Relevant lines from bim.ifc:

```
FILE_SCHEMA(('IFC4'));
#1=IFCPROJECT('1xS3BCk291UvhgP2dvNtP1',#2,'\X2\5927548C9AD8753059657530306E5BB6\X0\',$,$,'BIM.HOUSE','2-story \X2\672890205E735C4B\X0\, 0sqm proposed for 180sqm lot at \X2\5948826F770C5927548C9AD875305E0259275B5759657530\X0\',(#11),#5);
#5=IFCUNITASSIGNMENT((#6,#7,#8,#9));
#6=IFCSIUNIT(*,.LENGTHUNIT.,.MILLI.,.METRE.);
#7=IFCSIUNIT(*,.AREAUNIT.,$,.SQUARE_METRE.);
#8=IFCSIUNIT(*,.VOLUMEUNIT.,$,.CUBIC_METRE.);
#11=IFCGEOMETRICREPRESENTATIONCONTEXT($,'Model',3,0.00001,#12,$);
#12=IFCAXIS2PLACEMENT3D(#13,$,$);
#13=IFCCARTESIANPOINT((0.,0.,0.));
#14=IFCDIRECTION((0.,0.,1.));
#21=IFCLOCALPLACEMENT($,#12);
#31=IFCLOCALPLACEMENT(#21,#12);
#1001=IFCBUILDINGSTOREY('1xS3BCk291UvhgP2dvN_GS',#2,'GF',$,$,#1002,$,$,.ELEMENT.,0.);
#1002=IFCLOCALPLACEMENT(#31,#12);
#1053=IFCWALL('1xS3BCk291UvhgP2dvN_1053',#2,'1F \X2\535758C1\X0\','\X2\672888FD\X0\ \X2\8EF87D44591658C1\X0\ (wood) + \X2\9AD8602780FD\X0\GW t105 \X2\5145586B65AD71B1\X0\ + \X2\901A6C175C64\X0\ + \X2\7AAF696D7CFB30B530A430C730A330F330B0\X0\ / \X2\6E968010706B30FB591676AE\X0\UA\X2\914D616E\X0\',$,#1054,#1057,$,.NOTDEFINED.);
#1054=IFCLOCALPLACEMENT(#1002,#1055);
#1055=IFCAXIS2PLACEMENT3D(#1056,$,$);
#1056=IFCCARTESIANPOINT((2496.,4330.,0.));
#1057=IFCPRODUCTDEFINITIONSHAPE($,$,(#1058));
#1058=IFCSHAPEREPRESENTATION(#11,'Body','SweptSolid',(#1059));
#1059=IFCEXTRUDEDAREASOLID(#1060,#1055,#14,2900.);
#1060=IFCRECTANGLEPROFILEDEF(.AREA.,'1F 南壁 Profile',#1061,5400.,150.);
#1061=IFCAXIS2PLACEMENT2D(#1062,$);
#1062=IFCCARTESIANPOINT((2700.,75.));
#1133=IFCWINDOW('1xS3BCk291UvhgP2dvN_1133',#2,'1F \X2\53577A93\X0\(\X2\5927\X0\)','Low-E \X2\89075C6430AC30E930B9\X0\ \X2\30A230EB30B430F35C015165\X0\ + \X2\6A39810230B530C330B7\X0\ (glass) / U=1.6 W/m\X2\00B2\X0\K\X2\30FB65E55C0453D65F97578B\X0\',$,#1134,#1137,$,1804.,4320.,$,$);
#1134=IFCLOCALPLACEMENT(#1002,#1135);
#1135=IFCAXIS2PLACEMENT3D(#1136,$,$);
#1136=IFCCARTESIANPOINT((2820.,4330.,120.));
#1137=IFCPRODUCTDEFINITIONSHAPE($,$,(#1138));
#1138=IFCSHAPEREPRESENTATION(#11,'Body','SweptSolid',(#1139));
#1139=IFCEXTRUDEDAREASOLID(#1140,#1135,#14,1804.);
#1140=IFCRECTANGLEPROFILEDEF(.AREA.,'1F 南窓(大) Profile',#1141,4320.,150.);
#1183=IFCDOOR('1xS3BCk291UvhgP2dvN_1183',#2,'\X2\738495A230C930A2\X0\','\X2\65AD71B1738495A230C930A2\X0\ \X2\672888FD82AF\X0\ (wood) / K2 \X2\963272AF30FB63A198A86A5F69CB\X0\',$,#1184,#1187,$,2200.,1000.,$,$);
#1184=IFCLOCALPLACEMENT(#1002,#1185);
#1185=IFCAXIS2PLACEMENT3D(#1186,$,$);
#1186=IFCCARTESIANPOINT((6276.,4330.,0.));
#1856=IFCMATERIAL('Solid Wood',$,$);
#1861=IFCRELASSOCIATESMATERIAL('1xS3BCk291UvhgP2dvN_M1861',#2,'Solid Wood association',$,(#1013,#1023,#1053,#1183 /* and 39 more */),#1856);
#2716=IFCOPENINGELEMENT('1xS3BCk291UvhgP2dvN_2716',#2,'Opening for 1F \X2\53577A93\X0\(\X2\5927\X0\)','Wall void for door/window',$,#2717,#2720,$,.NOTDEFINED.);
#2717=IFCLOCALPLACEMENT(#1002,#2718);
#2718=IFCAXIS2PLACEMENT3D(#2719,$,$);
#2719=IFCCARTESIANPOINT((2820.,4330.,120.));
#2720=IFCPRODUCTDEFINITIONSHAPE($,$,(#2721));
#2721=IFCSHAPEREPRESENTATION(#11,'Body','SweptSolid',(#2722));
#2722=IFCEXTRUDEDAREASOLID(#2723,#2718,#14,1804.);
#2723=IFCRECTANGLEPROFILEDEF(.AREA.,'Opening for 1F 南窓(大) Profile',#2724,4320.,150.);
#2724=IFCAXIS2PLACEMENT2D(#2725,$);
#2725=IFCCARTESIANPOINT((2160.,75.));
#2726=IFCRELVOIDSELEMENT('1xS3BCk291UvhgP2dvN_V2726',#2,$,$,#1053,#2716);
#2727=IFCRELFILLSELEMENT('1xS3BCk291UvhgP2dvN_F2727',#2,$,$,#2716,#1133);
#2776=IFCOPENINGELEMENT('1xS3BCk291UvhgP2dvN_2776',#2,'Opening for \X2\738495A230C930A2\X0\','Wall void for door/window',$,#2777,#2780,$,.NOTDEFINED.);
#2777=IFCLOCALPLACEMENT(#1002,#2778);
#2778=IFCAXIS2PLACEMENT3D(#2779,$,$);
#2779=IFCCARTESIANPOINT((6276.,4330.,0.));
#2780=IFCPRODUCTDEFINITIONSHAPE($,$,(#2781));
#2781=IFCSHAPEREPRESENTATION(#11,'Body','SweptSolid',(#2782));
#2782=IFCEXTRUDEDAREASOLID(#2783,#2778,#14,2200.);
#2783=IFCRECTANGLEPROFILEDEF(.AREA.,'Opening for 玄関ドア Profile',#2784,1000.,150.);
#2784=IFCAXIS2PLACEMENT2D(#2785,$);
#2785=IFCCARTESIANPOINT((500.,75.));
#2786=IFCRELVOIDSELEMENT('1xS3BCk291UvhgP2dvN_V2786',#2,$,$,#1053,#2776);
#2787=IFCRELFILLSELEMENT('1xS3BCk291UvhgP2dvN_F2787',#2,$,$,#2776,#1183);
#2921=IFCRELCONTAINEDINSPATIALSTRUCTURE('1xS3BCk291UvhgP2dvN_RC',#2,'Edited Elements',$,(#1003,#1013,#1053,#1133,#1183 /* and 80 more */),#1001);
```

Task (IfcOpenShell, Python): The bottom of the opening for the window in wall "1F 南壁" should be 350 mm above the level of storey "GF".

```python
import numpy as np
import ifcopenshell
import ifcopenshell.api.geometry
import ifcopenshell.geom
import ifcopenshell.util.element
import ifcopenshell.util.placement
import ifcopenshell.util.shape
import ifcopenshell.util.unit

model = ifcopenshell.open("bim.ifc")
unit_scale = ifcopenshell.util.unit.calculate_unit_scale(model)

window = model.by_guid("1xS3BCk291UvhgP2dvN_1133")
opening = window.FillsVoids[0].RelatingOpeningElement
storey = ifcopenshell.util.element.get_container(window, ifc_class="IfcBuildingStorey")
level = ifcopenshell.util.placement.get_local_placement(storey.ObjectPlacement)[2, 3]

# The opening's origin need not be at the sill, so measure its lowest point.
shape = ifcopenshell.geom.create_shape(ifcopenshell.geom.settings(), opening)
bottom = ifcopenshell.util.shape.get_shape_bottom_elevation(shape, shape.geometry) / unit_scale
dz = level + 0.35 / unit_scale - bottom

shift = np.array([0.0, 0.0, dz])
# The window is not placed relative to its opening, so move both.
for product in (opening, window):
    matrix = ifcopenshell.util.placement.get_local_placement(product.ObjectPlacement)
    matrix[:3, 3] += shift
    ifcopenshell.api.geometry.edit_object_placement(model, product=product, matrix=matrix, is_si=False)

print(f"moved by {dz * unit_scale:+.3f} m")

model.write("bim-out.ifc")
```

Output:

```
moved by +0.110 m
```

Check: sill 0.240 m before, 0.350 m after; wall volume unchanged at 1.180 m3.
